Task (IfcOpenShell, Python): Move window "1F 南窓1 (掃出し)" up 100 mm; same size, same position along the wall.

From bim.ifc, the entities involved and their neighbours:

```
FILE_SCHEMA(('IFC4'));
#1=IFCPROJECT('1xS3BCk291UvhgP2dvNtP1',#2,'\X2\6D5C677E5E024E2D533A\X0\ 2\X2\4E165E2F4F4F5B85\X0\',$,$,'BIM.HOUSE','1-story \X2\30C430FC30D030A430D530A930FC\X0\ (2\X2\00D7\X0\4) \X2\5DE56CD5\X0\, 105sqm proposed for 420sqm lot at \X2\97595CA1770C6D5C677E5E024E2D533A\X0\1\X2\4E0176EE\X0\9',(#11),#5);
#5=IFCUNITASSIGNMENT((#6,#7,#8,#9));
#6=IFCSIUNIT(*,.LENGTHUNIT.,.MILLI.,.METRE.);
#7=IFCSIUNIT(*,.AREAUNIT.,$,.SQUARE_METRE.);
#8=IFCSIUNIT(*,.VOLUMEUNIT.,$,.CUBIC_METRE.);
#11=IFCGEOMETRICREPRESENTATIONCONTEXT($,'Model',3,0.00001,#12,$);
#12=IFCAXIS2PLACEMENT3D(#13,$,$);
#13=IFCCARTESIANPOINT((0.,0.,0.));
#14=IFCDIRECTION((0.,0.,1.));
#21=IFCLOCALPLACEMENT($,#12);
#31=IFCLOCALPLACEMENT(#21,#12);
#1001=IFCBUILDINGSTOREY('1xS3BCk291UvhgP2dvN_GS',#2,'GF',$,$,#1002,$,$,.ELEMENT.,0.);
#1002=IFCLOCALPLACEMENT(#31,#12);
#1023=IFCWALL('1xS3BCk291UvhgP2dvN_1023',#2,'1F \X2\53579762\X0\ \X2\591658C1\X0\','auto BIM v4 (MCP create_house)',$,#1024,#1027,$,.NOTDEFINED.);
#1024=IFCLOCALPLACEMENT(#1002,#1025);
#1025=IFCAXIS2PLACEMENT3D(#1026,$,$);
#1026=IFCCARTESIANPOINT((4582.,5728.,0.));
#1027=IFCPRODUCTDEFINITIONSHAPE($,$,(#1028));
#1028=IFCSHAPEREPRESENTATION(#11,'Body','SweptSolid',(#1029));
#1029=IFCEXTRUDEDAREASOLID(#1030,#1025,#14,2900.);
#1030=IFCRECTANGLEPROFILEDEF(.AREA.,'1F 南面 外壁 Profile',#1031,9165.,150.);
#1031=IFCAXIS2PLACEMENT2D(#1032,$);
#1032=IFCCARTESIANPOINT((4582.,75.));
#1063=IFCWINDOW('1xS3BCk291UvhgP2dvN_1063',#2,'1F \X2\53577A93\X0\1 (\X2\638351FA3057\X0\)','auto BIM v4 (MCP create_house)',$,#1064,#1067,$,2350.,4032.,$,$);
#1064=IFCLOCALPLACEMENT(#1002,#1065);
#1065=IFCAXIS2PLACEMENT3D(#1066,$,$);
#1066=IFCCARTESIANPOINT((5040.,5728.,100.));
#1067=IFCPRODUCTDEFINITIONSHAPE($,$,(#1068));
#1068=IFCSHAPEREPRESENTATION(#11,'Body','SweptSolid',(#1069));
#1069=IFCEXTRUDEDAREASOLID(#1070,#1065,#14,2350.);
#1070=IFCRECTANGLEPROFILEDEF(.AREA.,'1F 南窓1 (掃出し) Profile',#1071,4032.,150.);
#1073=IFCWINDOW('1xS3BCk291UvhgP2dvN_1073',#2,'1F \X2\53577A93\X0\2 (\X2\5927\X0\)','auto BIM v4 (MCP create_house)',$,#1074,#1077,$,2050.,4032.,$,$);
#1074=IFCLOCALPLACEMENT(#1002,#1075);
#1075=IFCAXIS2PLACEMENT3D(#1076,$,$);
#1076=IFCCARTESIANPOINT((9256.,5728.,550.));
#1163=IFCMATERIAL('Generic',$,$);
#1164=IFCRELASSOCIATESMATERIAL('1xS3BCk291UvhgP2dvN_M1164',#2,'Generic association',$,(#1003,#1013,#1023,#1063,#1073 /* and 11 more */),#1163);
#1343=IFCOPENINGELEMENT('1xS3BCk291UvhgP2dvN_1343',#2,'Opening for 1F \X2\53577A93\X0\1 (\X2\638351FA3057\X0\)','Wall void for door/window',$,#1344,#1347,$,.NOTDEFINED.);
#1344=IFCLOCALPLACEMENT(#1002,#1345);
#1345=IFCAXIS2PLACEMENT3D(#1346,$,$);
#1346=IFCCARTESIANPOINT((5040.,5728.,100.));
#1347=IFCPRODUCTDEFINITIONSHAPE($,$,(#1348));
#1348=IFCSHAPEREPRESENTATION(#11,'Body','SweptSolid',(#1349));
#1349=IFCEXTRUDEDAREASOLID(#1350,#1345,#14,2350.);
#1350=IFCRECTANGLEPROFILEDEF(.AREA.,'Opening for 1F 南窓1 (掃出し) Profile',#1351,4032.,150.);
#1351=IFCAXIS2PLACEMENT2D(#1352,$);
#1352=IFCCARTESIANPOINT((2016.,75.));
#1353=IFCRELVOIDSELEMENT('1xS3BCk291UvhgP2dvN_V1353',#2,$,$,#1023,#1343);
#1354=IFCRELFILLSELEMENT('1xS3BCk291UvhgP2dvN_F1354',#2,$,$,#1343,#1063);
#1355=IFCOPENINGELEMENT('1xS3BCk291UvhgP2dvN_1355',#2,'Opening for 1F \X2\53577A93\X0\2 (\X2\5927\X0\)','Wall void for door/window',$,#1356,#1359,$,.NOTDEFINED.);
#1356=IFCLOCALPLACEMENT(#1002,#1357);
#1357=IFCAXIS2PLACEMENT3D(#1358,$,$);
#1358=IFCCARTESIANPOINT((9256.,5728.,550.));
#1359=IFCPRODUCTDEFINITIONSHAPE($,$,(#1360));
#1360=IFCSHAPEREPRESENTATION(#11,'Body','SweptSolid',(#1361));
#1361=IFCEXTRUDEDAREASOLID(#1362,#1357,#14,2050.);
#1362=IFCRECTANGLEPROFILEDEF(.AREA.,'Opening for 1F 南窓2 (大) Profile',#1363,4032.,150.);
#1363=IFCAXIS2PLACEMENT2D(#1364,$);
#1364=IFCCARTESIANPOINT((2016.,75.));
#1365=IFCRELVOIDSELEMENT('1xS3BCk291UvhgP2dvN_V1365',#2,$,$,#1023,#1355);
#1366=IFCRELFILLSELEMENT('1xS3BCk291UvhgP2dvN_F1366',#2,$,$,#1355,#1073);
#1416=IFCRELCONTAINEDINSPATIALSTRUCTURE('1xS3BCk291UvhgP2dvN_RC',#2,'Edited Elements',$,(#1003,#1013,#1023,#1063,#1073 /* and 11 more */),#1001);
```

```python
import numpy as np
import ifcopenshell
import ifcopenshell.api.geometry
import ifcopenshell.util.placement
import ifcopenshell.util.unit

model = ifcopenshell.open("bim.ifc")
unit_scale = ifcopenshell.util.unit.calculate_unit_scale(model)

window = model.by_id(1063)
opening = window.FillsVoids[0].RelatingOpeningElement
dz = 100.0

shift = np.array([0.0, 0.0, dz])
# The window is not placed relative to its opening, so move both.
for product in (opening, window):
    matrix = ifcopenshell.util.placement.get_local_placement(product.ObjectPlacement)
    matrix[:3, 3] += shift
    ifcopenshell.api.geometry.edit_object_placement(model, product=product, matrix=matrix, is_si=False)

print(f"moved by {dz * unit_scale:+.3f} m")

model.write("bim_v2.ifc")
```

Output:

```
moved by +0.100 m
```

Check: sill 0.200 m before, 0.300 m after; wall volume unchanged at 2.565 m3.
